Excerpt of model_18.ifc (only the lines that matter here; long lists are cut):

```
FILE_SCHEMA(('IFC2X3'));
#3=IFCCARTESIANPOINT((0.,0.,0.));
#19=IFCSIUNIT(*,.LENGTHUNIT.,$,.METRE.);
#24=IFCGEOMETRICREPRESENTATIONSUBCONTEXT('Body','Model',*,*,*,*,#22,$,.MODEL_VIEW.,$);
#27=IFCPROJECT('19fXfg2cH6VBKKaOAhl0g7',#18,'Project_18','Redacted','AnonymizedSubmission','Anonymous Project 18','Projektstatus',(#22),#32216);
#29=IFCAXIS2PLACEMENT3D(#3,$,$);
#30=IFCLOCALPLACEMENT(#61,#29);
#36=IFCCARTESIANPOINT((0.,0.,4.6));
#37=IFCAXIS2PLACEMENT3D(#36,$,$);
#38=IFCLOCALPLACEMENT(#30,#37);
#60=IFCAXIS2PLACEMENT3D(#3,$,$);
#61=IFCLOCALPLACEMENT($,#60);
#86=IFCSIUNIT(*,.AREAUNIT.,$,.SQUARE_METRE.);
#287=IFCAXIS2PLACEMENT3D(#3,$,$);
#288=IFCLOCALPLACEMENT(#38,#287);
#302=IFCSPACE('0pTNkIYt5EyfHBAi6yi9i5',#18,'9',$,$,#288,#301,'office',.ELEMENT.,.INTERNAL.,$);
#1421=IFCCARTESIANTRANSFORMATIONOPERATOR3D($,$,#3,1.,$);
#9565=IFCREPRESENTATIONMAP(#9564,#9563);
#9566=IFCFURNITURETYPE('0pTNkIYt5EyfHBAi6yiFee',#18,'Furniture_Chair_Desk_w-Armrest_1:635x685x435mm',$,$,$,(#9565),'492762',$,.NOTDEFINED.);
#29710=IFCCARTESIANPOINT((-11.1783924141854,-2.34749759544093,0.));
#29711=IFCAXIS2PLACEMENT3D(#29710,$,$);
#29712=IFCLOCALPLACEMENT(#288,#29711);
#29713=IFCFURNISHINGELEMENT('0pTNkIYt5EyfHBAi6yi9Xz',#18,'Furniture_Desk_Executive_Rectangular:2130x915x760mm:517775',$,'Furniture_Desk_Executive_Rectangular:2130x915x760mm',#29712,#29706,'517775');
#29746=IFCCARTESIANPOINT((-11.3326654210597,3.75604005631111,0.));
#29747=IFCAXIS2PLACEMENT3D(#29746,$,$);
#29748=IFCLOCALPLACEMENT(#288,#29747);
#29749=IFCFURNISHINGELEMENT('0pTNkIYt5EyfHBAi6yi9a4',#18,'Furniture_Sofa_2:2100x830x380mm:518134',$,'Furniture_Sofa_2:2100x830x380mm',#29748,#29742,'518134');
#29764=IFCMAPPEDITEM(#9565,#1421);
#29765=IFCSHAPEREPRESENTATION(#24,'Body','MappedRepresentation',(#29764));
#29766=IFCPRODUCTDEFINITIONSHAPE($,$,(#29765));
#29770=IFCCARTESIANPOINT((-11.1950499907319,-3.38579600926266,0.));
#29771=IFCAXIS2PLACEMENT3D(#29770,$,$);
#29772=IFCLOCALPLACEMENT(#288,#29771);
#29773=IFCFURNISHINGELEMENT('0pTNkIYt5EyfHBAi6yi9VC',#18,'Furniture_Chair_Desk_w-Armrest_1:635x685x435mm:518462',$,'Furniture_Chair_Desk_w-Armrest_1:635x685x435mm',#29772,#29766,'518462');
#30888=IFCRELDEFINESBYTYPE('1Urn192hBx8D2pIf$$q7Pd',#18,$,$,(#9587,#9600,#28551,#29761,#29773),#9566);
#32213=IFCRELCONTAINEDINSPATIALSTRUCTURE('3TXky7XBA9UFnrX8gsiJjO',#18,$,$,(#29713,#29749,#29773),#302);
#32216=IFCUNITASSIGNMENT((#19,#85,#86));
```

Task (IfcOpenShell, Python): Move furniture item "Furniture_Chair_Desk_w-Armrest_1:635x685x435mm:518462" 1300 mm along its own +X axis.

```python
import ifcopenshell
import ifcopenshell.api.geometry
import ifcopenshell.util.placement
import ifcopenshell.util.unit

model = ifcopenshell.open("model_18.ifc")
unit_scale = ifcopenshell.util.unit.calculate_unit_scale(model)

item = model.by_guid("0pTNkIYt5EyfHBAi6yi9VC")
matrix = ifcopenshell.util.placement.get_local_placement(item.ObjectPlacement)
matrix[:3, 3] += matrix[:3, 0] * 1.3 / unit_scale
ifcopenshell.api.geometry.edit_object_placement(model, product=item, matrix=matrix, is_si=False)

print(ifcopenshell.util.placement.get_local_placement(item.ObjectPlacement).round(3) + 0.0)

model.write("model_18_rev.ifc")
```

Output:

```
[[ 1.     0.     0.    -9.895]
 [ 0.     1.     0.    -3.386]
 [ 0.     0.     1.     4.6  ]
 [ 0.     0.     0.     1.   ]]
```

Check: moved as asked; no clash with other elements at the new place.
